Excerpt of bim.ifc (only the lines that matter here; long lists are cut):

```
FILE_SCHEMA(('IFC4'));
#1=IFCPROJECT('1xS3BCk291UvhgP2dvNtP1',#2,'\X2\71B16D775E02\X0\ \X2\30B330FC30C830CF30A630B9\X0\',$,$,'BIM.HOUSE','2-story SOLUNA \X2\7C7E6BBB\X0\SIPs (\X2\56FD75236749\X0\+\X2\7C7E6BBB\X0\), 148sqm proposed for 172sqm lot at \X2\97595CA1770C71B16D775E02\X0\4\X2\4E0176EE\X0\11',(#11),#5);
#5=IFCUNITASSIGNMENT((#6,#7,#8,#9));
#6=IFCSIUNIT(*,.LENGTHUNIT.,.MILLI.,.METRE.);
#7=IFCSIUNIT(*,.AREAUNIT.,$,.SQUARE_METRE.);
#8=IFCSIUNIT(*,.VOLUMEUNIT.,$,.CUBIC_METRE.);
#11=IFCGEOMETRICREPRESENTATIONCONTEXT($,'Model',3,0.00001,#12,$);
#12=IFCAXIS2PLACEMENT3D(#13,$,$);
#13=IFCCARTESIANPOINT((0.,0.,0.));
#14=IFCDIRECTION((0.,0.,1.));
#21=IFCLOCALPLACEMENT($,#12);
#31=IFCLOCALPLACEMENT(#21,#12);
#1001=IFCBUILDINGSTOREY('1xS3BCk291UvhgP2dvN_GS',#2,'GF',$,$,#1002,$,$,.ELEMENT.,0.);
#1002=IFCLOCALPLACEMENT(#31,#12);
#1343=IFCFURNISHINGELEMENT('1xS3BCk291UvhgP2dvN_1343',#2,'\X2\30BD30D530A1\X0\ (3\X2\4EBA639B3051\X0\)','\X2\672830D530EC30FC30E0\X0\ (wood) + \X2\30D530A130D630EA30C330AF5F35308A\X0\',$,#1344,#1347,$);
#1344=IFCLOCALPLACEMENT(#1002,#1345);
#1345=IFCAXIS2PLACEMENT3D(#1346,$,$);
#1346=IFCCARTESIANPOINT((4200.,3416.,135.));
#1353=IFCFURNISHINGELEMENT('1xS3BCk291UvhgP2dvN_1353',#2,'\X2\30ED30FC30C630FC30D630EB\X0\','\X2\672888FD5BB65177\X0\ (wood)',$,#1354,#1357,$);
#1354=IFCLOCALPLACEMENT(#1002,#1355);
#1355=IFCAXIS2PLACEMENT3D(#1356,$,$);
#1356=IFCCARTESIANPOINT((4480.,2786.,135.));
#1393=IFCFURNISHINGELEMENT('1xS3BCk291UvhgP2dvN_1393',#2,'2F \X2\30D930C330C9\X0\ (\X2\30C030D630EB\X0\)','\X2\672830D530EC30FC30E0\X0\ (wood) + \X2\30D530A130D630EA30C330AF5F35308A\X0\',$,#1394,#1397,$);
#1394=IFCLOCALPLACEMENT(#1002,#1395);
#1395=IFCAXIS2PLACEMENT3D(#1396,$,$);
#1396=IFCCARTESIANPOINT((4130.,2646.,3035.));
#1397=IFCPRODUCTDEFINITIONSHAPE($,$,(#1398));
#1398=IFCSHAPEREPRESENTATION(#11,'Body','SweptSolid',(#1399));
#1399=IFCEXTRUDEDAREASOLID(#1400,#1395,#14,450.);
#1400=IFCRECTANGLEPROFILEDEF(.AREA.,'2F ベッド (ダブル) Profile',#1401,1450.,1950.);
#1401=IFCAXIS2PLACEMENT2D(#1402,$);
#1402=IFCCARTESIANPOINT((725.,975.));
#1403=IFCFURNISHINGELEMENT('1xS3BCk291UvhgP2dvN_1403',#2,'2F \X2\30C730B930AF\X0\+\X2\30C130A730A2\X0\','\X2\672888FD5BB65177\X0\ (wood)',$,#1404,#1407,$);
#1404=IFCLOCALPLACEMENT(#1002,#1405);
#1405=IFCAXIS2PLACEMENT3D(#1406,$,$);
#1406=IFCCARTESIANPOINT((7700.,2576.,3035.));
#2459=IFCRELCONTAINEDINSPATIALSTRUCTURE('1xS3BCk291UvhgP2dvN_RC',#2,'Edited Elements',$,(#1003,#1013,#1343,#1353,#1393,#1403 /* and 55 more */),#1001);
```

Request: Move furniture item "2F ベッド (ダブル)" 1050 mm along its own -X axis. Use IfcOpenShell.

```python
import ifcopenshell
import ifcopenshell.api.geometry
import ifcopenshell.util.placement
import ifcopenshell.util.unit

model = ifcopenshell.open("bim.ifc")
unit_scale = ifcopenshell.util.unit.calculate_unit_scale(model)

item = model.by_guid("1xS3BCk291UvhgP2dvN_1393")
matrix = ifcopenshell.util.placement.get_local_placement(item.ObjectPlacement)
matrix[:3, 3] -= matrix[:3, 0] * 1.05 / unit_scale
ifcopenshell.api.geometry.edit_object_placement(model, product=item, matrix=matrix, is_si=False)

print(ifcopenshell.util.placement.get_local_placement(item.ObjectPlacement).round(3) + 0.0)

model.write("bim_v2.ifc")
```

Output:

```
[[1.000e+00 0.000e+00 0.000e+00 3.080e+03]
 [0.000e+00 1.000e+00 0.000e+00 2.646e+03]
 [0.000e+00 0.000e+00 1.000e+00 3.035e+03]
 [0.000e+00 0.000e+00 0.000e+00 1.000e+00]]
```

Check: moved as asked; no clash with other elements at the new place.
